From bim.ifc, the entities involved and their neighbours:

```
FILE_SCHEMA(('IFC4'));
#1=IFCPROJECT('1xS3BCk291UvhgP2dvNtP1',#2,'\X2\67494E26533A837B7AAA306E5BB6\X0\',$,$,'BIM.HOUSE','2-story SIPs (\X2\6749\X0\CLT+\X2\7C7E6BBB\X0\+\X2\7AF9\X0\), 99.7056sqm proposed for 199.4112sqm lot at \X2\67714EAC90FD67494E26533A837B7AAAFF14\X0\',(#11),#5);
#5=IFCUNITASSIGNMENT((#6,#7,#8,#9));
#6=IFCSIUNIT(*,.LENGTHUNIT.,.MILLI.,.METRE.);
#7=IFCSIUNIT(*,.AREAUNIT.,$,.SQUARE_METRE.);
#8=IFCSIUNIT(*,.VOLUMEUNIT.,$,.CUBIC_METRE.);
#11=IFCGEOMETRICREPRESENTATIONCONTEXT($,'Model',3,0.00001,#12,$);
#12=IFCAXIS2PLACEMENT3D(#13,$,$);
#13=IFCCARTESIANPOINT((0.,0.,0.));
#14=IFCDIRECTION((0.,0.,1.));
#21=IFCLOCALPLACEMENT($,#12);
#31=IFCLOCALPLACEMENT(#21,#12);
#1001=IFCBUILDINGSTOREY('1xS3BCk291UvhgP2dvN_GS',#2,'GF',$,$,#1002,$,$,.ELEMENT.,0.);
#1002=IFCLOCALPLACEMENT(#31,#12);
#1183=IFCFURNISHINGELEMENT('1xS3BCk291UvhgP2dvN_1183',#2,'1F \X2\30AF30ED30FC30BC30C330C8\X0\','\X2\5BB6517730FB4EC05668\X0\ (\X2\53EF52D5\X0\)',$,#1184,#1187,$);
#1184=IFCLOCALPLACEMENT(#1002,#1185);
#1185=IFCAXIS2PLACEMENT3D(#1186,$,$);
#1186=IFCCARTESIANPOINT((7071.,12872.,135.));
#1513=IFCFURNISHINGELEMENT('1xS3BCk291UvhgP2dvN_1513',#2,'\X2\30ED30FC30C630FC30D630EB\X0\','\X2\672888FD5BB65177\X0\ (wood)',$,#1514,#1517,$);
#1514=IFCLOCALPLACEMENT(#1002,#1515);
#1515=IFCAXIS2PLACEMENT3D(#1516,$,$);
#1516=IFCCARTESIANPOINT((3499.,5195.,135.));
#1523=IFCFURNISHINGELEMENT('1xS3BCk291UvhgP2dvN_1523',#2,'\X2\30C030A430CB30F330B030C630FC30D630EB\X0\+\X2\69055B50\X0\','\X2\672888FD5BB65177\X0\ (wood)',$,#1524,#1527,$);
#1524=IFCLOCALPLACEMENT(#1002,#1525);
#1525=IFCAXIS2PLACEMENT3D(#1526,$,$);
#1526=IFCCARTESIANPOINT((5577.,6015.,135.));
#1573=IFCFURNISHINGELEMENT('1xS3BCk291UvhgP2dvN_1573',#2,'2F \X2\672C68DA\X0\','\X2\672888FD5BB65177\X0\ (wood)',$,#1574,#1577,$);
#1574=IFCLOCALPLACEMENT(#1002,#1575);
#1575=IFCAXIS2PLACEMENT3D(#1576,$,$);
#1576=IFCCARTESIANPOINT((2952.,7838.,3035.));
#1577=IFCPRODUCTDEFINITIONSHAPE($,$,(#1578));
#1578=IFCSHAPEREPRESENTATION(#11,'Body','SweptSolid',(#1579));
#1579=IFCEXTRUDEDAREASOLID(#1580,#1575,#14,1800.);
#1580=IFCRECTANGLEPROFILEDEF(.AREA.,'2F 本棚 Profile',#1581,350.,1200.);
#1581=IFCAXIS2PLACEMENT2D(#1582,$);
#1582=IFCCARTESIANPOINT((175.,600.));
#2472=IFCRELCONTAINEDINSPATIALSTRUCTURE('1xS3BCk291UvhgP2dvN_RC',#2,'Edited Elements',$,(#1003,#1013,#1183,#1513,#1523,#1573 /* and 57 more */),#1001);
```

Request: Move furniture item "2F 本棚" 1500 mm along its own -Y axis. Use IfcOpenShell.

```python
import ifcopenshell
import ifcopenshell.api.geometry
import ifcopenshell.util.placement
import ifcopenshell.util.unit

model = ifcopenshell.open("bim.ifc")
unit_scale = ifcopenshell.util.unit.calculate_unit_scale(model)

item = model.by_id(1573)
matrix = ifcopenshell.util.placement.get_local_placement(item.ObjectPlacement)
matrix[:3, 3] -= matrix[:3, 1] * 1.5 / unit_scale
ifcopenshell.api.geometry.edit_object_placement(model, product=item, matrix=matrix, is_si=False)

print(ifcopenshell.util.placement.get_local_placement(item.ObjectPlacement).round(3) + 0.0)

model.write("bim_v2.ifc")
```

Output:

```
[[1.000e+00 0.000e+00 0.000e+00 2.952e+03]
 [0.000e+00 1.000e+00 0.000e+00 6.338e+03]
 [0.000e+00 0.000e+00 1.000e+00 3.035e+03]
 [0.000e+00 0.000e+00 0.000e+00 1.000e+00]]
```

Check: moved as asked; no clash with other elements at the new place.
